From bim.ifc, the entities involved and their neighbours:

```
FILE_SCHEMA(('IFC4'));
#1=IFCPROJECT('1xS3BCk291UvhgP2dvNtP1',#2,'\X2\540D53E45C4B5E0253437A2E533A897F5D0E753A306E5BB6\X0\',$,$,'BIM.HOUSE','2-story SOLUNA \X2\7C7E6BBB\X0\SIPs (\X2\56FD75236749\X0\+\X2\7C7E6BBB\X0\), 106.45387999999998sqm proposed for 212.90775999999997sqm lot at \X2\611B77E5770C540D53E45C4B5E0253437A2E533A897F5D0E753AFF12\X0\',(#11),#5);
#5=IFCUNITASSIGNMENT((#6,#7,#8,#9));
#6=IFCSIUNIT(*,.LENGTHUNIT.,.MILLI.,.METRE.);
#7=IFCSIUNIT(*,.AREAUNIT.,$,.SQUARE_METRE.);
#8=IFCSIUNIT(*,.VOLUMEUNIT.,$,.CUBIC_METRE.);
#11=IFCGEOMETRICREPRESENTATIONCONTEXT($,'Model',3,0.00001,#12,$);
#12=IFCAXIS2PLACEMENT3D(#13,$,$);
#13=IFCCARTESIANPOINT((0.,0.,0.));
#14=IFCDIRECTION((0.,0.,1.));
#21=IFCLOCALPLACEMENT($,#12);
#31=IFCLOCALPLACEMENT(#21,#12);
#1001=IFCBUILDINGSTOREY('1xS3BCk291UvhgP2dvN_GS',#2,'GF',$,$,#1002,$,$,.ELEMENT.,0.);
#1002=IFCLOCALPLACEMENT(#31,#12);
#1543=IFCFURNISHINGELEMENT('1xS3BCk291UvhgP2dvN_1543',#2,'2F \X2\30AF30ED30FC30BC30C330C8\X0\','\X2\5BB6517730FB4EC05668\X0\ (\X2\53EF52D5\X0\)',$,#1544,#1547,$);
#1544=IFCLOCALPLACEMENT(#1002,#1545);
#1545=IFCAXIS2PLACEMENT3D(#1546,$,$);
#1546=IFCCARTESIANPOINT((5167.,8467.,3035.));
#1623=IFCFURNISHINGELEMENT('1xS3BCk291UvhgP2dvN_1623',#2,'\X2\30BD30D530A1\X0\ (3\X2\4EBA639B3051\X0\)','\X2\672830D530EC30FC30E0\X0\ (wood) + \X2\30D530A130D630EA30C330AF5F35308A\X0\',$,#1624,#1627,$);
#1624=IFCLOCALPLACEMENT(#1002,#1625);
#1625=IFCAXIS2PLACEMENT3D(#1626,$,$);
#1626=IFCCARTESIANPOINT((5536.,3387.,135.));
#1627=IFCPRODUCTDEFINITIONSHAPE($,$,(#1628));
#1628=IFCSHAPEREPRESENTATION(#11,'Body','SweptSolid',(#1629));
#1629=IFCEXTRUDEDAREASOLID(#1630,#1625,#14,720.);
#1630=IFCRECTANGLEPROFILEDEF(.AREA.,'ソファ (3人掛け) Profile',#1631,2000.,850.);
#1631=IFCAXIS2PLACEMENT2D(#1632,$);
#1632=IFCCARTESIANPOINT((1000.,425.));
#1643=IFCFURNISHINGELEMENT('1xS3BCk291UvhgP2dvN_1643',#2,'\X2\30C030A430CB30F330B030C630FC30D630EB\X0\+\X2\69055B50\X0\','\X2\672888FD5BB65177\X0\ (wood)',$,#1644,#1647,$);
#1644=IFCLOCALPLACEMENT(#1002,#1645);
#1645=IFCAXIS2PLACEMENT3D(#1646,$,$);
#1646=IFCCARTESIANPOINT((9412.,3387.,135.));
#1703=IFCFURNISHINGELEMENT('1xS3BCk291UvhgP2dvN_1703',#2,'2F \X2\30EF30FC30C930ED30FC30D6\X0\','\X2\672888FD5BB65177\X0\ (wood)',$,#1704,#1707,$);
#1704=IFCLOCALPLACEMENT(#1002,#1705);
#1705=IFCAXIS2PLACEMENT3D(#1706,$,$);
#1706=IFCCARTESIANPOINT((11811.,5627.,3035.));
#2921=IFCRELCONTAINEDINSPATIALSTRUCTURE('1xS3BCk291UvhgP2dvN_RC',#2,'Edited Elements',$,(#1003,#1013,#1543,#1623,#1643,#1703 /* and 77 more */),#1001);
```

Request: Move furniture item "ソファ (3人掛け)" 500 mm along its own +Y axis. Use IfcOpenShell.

```python
import ifcopenshell
import ifcopenshell.api.geometry
import ifcopenshell.util.placement
import ifcopenshell.util.unit

model = ifcopenshell.open("bim.ifc")
unit_scale = ifcopenshell.util.unit.calculate_unit_scale(model)

item = model.by_id(1623)
matrix = ifcopenshell.util.placement.get_local_placement(item.ObjectPlacement)
matrix[:3, 3] += matrix[:3, 1] * 0.5 / unit_scale
ifcopenshell.api.geometry.edit_object_placement(model, product=item, matrix=matrix, is_si=False)

print(ifcopenshell.util.placement.get_local_placement(item.ObjectPlacement).round(3) + 0.0)

model.write("bim_updated.ifc")
```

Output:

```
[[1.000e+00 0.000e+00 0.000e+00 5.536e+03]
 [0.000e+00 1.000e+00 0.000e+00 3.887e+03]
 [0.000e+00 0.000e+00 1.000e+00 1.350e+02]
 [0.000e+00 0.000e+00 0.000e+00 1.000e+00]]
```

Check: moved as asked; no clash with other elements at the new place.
